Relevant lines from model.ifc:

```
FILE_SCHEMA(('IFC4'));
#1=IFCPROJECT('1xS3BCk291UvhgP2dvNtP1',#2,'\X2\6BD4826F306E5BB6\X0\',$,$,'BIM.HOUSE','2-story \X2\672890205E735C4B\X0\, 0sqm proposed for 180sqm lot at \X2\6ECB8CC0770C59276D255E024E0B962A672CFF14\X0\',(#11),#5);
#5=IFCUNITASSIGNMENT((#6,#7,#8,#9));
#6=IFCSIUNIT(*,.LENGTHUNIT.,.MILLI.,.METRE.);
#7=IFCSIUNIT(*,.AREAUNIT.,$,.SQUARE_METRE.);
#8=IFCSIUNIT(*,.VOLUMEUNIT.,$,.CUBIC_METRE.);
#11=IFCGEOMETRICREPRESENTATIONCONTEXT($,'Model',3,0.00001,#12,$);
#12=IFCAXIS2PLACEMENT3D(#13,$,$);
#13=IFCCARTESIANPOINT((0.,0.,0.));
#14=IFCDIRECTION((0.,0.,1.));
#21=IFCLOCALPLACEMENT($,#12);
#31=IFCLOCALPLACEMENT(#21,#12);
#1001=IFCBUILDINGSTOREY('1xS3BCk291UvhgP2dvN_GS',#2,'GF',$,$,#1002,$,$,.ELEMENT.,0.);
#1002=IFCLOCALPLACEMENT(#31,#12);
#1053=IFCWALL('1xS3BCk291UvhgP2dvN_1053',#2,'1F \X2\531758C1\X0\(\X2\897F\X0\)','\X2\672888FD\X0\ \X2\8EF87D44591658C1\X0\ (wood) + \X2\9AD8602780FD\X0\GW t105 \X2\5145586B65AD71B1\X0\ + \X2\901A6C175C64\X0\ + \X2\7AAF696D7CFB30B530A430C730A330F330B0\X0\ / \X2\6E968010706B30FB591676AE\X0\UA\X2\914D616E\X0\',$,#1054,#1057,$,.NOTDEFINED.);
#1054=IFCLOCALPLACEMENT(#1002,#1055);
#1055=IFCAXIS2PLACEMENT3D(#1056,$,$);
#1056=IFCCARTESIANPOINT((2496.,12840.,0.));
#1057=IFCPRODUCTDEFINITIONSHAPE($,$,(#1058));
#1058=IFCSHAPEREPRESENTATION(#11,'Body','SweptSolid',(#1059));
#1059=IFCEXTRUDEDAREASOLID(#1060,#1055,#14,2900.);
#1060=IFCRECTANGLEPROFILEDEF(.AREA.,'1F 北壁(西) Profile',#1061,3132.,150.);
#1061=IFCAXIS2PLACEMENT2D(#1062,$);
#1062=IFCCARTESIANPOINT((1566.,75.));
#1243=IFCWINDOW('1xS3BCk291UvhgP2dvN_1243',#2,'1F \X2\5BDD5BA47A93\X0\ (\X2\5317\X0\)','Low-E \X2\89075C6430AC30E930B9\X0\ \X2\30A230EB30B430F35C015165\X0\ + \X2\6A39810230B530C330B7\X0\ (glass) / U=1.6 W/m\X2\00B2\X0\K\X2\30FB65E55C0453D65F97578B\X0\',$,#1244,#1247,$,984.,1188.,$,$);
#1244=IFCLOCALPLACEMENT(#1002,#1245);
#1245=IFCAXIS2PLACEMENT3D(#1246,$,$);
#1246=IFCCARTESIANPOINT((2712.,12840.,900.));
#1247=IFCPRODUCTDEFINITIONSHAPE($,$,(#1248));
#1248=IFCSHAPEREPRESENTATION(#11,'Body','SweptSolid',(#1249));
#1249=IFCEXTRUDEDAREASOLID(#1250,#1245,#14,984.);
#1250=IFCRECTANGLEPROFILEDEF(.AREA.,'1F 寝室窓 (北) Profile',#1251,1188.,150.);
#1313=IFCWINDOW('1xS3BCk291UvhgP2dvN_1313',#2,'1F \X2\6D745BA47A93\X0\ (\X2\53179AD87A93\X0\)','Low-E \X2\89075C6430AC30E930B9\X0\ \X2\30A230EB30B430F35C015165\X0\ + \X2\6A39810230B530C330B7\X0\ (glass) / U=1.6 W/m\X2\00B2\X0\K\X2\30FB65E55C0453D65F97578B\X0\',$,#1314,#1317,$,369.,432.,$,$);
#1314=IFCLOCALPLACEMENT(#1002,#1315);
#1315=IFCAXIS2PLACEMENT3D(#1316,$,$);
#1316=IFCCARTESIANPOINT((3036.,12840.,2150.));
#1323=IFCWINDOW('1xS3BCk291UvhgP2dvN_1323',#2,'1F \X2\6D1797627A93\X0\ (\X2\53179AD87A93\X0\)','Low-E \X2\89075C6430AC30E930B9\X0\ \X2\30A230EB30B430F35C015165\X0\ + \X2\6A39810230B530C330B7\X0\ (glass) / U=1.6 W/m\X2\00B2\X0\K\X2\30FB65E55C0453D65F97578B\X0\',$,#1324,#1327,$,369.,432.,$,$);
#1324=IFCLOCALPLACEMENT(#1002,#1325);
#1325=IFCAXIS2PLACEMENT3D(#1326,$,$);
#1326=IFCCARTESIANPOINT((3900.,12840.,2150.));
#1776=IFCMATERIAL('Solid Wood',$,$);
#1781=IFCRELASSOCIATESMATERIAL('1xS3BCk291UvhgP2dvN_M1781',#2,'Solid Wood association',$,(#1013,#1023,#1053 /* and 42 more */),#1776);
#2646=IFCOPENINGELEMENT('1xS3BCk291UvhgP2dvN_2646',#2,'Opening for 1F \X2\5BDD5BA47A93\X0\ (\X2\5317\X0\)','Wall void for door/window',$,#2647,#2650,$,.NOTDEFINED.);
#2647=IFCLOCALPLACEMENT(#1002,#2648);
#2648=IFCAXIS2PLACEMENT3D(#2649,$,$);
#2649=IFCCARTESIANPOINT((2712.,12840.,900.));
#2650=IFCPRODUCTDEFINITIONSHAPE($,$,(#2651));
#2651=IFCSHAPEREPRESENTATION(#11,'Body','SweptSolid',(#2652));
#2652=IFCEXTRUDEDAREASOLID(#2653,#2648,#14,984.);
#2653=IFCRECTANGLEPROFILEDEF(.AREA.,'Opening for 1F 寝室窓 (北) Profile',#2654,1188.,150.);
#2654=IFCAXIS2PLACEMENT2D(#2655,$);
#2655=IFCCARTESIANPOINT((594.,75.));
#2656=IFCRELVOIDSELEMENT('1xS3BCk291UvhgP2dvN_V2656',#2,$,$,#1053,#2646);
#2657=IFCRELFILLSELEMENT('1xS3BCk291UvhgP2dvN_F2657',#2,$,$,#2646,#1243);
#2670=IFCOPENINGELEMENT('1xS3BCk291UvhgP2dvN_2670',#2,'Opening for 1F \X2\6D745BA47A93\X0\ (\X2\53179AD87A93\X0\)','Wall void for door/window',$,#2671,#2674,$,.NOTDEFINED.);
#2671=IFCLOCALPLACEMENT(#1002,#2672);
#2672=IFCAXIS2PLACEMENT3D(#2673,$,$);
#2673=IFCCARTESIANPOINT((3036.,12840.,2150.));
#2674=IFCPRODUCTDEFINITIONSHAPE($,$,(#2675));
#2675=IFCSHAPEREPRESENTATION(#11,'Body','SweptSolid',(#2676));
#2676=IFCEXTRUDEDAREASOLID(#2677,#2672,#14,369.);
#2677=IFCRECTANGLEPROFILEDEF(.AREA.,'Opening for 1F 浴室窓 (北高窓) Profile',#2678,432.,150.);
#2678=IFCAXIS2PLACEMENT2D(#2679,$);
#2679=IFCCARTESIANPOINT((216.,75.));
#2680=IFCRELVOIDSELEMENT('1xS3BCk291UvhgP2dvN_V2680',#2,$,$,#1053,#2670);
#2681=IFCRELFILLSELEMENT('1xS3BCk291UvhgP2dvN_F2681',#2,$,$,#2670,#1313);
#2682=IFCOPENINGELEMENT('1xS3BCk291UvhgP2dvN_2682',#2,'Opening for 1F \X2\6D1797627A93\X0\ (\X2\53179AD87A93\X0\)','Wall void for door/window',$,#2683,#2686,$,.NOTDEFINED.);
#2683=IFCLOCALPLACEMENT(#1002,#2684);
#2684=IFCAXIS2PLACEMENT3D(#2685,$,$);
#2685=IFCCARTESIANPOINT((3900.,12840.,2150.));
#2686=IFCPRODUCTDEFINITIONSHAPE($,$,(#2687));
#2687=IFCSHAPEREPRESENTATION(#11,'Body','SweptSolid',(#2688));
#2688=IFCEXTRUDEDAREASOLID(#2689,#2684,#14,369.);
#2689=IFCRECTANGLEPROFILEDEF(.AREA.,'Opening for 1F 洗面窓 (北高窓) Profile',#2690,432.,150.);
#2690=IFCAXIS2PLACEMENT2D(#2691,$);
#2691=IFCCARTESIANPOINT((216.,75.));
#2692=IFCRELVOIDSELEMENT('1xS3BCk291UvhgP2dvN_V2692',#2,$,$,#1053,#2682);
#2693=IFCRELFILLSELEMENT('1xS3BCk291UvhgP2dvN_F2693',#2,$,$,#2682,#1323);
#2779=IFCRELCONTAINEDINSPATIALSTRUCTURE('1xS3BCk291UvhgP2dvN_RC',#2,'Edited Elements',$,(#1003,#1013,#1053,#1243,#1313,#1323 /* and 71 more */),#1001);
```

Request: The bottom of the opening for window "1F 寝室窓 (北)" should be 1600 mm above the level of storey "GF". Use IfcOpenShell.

```python
import numpy as np
import ifcopenshell
import ifcopenshell.api.geometry
import ifcopenshell.geom
import ifcopenshell.util.element
import ifcopenshell.util.placement
import ifcopenshell.util.shape
import ifcopenshell.util.unit

model = ifcopenshell.open("model.ifc")
unit_scale = ifcopenshell.util.unit.calculate_unit_scale(model)

window = model.by_guid("1xS3BCk291UvhgP2dvN_1243")
opening = window.FillsVoids[0].RelatingOpeningElement
storey = ifcopenshell.util.element.get_container(window, ifc_class="IfcBuildingStorey")
level = ifcopenshell.util.placement.get_local_placement(storey.ObjectPlacement)[2, 3]

# The opening's origin need not be at the sill, so measure its lowest point.
shape = ifcopenshell.geom.create_shape(ifcopenshell.geom.settings(), opening)
bottom = ifcopenshell.util.shape.get_shape_bottom_elevation(shape, shape.geometry) / unit_scale
dz = level + 1600.0 - bottom

shift = np.array([0.0, 0.0, dz])
# The window is not placed relative to its opening, so move both.
for product in (opening, window):
    matrix = ifcopenshell.util.placement.get_local_placement(product.ObjectPlacement)
    matrix[:3, 3] += shift
    ifcopenshell.api.geometry.edit_object_placement(model, product=product, matrix=matrix, is_si=False)

print(f"moved by {dz * unit_scale:+.3f} m")

model.write("model_v2.ifc")
```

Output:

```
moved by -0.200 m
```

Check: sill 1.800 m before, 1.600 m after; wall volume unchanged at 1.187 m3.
